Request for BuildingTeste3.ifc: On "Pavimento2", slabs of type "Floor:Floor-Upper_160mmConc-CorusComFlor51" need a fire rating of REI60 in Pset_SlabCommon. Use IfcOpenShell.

First a look at what the model holds.

```python
import ifcopenshell
import ifcopenshell.util.element

model = ifcopenshell.open("BuildingTeste3.ifc")
print(model.schema)
storey = next(s for s in model.by_type("IfcBuildingStorey") if s.Name == "Pavimento2")
slabs = [e for e in ifcopenshell.util.element.get_decomposition(storey) if e.is_a("IfcSlab")]
seen = {}
for e in slabs:
    element_type = ifcopenshell.util.element.get_type(e)
    key = (element_type.Name if element_type != e and element_type else None, ifcopenshell.util.element.get_pset(e, "Pset_SlabCommon", "FireRating"))
    seen[key] = seen.get(key, 0) + 1
for (name, value), count in sorted(seen.items(), key=str):
    print(count, "x", name, "|", value)
```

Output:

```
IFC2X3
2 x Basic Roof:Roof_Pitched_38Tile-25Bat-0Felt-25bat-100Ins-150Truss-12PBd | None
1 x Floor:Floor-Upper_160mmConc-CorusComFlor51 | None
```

```python
import ifcopenshell
import ifcopenshell.api.pset
import ifcopenshell.util.element

model = ifcopenshell.open("BuildingTeste3.ifc")

storey = next(s for s in model.by_type("IfcBuildingStorey") if s.Name == "Pavimento2")
slabs = [e for e in ifcopenshell.util.element.get_decomposition(storey) if e.is_a("IfcSlab")]

count = 0
for e in slabs:
    element_type = ifcopenshell.util.element.get_type(e)
    if element_type in (None, e) or element_type.Name != "Floor:Floor-Upper_160mmConc-CorusComFlor51":
        continue
    # add_pset returns the element's existing set when there is one.
    pset = ifcopenshell.api.pset.add_pset(model, product=e, name="Pset_SlabCommon")
    ifcopenshell.api.pset.edit_pset(model, pset=pset, properties={"FireRating": "REI60"})
    count += 1

print(count, "slabs updated")

model.write("BuildingTeste3-out.ifc")
```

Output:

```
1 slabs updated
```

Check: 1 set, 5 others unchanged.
